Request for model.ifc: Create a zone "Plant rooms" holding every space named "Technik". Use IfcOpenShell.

First a look at what the model holds.

```python
import ifcopenshell

model = ifcopenshell.open("model.ifc")
print(model.schema)
seen = {}
for space in model.by_type("IfcSpace"):
    seen[space.LongName] = seen.get(space.LongName, 0) + 1
for name, count in sorted(seen.items(), key=str):
    print(count, "x", name)
print("zones:", [z.Name for z in model.by_type("IfcZone")][:20])
```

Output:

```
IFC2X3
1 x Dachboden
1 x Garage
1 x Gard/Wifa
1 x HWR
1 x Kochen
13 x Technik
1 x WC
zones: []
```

```python
import ifcopenshell
import ifcopenshell.api.group
import ifcopenshell.api.root

model = ifcopenshell.open("model.ifc")

names = {"Technik"}
spaces = [s for s in model.by_type("IfcSpace") if s.LongName in names]

zone = ifcopenshell.api.root.create_entity(model, ifc_class="IfcZone", name="Plant rooms")
ifcopenshell.api.group.assign_group(model, products=spaces, group=zone)
print(len(spaces), "spaces in", zone.Name)

model.write("model_edited.ifc")
```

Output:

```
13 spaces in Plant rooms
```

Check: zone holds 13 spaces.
